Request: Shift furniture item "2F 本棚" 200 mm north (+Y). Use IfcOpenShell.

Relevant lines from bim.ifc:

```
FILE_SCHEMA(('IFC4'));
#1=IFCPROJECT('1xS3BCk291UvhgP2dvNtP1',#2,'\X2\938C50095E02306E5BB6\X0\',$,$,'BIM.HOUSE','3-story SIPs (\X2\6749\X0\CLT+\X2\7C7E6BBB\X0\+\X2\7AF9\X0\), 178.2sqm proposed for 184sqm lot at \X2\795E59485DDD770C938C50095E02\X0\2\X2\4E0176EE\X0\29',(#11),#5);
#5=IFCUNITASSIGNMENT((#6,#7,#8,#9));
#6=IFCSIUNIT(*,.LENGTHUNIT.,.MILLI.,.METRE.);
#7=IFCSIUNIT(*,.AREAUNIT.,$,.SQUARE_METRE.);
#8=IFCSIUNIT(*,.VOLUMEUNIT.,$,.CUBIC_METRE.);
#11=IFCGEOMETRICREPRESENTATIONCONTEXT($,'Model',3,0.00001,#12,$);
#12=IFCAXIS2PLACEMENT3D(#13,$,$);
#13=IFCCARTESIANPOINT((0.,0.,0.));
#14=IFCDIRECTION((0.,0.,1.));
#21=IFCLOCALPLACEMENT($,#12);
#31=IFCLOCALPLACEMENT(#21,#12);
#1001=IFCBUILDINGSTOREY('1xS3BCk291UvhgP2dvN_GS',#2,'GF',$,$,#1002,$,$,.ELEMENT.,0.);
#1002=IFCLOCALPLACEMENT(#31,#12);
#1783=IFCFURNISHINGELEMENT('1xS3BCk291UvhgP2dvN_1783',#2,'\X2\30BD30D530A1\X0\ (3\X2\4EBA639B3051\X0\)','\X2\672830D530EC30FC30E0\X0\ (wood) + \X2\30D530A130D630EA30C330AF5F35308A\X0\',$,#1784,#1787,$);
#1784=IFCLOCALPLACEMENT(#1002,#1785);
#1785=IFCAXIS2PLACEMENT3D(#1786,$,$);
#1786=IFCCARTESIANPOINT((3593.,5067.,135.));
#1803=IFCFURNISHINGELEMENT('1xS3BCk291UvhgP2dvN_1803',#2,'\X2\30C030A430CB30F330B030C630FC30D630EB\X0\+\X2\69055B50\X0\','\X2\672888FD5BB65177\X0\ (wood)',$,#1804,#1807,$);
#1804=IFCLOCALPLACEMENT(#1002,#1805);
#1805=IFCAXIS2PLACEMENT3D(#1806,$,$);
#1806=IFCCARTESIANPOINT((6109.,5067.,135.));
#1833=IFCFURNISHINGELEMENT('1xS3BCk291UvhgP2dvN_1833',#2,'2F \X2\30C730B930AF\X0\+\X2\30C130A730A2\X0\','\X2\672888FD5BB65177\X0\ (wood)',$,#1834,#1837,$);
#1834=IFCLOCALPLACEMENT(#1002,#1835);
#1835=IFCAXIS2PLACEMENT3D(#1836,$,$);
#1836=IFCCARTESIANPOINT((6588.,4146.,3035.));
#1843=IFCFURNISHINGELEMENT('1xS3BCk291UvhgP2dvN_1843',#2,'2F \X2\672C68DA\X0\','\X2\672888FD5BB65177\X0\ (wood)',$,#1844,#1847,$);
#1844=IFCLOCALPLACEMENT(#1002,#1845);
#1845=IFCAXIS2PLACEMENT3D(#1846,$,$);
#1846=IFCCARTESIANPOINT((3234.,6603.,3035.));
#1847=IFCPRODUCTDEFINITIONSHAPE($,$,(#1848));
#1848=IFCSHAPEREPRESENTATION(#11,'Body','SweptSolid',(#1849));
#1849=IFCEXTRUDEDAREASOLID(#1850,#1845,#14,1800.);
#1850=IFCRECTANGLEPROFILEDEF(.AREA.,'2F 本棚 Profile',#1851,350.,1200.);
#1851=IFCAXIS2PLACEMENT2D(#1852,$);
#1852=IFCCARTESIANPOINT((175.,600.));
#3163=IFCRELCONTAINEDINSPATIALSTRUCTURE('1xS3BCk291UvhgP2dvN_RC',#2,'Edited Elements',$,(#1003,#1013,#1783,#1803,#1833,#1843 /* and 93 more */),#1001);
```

```python
import ifcopenshell
import ifcopenshell.api.geometry
import ifcopenshell.util.placement

model = ifcopenshell.open("bim.ifc")

item = model.by_guid("1xS3BCk291UvhgP2dvN_1843")
matrix = ifcopenshell.util.placement.get_local_placement(item.ObjectPlacement)
matrix[1, 3] += 200.0
ifcopenshell.api.geometry.edit_object_placement(model, product=item, matrix=matrix, is_si=False)

print(ifcopenshell.util.placement.get_local_placement(item.ObjectPlacement).round(3) + 0.0)

model.write("bim_rev.ifc")
```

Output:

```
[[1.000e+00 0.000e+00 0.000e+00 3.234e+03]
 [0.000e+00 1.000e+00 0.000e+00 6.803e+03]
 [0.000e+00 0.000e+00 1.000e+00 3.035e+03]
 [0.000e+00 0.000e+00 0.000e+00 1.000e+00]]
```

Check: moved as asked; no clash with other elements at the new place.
